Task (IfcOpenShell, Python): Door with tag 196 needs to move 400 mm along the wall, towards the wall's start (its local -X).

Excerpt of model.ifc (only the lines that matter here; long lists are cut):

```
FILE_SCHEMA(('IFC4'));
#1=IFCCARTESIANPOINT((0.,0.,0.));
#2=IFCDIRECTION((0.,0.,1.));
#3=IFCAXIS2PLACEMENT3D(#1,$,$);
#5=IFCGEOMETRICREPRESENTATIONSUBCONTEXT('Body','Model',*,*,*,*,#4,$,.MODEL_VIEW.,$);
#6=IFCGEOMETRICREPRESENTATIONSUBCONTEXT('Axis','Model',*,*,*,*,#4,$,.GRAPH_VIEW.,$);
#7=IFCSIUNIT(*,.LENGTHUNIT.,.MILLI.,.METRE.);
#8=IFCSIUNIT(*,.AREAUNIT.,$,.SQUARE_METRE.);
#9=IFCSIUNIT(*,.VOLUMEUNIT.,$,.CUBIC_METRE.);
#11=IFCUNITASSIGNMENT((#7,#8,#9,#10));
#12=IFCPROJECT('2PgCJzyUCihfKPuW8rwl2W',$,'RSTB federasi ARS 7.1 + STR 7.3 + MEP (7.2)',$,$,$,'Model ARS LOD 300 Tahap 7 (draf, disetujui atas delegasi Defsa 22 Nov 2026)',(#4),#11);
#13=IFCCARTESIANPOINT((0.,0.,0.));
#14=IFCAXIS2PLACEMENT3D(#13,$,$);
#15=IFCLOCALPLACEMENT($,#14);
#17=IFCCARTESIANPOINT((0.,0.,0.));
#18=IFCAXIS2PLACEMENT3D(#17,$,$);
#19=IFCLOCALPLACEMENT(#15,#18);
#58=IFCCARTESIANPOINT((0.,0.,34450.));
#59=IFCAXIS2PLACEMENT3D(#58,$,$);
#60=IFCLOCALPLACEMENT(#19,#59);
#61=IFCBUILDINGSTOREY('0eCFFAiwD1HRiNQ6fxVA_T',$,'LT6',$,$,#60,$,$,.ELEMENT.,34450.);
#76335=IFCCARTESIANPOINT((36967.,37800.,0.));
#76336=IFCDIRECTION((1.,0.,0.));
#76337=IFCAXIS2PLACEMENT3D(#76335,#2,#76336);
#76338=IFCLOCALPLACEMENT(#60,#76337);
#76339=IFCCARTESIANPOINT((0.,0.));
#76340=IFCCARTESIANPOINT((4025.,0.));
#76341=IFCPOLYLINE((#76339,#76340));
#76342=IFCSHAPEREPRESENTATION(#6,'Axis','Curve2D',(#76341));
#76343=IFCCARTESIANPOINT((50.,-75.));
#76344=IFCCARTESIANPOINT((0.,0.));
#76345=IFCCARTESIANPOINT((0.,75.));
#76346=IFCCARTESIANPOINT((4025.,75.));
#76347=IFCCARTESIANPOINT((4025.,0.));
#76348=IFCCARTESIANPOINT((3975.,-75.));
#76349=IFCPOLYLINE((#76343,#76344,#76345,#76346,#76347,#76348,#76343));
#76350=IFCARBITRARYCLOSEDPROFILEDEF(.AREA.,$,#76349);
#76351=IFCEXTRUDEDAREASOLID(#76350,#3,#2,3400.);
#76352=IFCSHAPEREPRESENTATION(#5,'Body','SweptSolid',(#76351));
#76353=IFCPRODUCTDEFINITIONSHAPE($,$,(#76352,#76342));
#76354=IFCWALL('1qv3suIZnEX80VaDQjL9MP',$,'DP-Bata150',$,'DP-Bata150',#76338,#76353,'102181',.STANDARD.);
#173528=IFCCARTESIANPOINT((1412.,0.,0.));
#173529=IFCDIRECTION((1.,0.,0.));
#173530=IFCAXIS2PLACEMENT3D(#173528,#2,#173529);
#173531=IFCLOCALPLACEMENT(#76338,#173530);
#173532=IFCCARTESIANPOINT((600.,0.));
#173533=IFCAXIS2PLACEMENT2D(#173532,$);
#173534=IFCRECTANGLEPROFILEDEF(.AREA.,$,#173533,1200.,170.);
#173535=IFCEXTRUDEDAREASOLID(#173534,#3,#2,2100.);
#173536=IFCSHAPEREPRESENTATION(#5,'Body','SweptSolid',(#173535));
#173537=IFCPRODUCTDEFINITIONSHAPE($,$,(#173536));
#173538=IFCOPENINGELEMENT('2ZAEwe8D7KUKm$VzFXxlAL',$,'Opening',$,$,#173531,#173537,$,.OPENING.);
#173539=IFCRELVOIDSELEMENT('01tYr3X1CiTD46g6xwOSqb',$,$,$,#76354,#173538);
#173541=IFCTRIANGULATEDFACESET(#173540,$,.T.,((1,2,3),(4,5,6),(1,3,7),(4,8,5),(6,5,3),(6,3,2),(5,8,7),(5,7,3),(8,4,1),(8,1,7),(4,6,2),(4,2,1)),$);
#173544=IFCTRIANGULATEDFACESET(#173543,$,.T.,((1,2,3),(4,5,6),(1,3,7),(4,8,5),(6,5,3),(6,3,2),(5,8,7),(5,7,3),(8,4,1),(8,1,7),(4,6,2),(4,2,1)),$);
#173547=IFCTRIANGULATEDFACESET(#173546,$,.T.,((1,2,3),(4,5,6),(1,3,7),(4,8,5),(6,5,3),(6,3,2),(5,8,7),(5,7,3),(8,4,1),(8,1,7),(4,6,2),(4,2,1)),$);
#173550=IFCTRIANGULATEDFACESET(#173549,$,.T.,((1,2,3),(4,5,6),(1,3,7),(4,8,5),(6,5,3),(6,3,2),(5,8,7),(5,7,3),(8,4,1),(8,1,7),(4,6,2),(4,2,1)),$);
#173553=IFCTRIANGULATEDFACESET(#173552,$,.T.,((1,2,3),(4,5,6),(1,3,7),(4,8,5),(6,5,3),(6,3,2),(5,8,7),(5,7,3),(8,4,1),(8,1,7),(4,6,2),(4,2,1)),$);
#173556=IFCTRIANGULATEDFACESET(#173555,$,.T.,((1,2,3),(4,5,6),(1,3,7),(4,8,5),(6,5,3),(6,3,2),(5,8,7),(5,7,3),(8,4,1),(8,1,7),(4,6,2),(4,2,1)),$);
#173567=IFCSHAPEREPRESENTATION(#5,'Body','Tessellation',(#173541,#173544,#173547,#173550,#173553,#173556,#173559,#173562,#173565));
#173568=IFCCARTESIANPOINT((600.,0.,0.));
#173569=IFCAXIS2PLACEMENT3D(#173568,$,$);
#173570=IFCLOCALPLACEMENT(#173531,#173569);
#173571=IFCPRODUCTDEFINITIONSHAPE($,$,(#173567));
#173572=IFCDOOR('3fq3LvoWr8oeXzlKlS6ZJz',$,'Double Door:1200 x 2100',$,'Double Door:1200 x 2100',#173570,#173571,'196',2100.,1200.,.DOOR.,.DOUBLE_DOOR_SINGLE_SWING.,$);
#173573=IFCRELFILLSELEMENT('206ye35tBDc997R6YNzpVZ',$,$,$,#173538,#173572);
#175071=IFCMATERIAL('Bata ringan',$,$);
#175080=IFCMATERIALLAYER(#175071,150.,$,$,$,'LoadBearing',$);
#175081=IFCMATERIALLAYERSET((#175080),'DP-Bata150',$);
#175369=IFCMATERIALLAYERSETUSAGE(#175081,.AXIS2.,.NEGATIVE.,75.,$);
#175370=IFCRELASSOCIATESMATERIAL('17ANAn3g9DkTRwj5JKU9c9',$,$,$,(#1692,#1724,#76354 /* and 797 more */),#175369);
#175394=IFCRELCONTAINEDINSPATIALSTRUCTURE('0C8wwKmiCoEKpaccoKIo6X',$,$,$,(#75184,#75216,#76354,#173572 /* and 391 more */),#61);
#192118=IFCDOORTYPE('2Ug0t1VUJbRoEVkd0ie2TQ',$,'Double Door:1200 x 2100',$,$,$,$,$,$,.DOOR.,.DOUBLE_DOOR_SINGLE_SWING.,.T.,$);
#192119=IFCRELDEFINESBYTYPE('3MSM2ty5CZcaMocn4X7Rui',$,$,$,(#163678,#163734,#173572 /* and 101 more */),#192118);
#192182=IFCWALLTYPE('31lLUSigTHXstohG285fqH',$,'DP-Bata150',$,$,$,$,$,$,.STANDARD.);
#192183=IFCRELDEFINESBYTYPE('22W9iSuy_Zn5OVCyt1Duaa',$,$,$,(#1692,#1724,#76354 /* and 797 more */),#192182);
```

```python
import ifcopenshell
import ifcopenshell.api.geometry
import ifcopenshell.util.placement
import ifcopenshell.util.unit

model = ifcopenshell.open("model.ifc")
unit_scale = ifcopenshell.util.unit.calculate_unit_scale(model)

door = model.by_id(173572)
opening = door.FillsVoids[0].RelatingOpeningElement
wall = opening.VoidsElements[0].RelatingBuildingElement

wall_matrix = ifcopenshell.util.placement.get_local_placement(wall.ObjectPlacement)
shift = wall_matrix[:3, 0] * -0.4 / unit_scale
before = ifcopenshell.util.placement.get_local_placement(door.ObjectPlacement)[:3, 3].copy()

# The door is placed relative to its opening, so it follows when the opening moves.
matrix = ifcopenshell.util.placement.get_local_placement(opening.ObjectPlacement)
matrix[:3, 3] += shift
ifcopenshell.api.geometry.edit_object_placement(
    model, product=opening, matrix=matrix, is_si=False, should_transform_children=True
)

after = ifcopenshell.util.placement.get_local_placement(door.ObjectPlacement)[:3, 3]
print("door moved by", (after - before).round(3) + 0.0)

model.write("model_updated.ifc")
```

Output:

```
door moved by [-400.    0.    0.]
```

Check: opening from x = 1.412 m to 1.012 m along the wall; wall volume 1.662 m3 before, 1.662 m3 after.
